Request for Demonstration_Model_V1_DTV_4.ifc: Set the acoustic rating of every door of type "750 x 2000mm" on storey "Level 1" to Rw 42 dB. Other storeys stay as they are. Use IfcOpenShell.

First a look at what the model holds.

```python
import ifcopenshell
import ifcopenshell.util.element

model = ifcopenshell.open("Demonstration_Model_V1_DTV_4.ifc")
print(model.schema)
storey = next(s for s in model.by_type("IfcBuildingStorey") if s.Name == "Level 1")
doors = [e for e in ifcopenshell.util.element.get_decomposition(storey) if e.is_a("IfcDoor")]
seen = {}
for e in doors:
    element_type = ifcopenshell.util.element.get_type(e)
    key = (element_type.Name if element_type != e and element_type else None, ifcopenshell.util.element.get_pset(e, "Pset_DoorCommon", "AcousticRating"))
    seen[key] = seen.get(key, 0) + 1
for (name, value), count in sorted(seen.items(), key=str):
    print(count, "x", name, "|", value)
```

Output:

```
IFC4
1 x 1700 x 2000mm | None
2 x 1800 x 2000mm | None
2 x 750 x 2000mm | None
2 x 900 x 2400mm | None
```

```python
import ifcopenshell
import ifcopenshell.api.pset
import ifcopenshell.util.element

model = ifcopenshell.open("Demonstration_Model_V1_DTV_4.ifc")

storey = next(s for s in model.by_type("IfcBuildingStorey") if s.Name == "Level 1")
doors = [e for e in ifcopenshell.util.element.get_decomposition(storey) if e.is_a("IfcDoor")]

count = 0
for e in doors:
    element_type = ifcopenshell.util.element.get_type(e)
    if element_type in (None, e) or element_type.Name != "750 x 2000mm":
        continue
    # add_pset returns the element's existing set when there is one.
    pset = ifcopenshell.api.pset.add_pset(model, product=e, name="Pset_DoorCommon")
    ifcopenshell.api.pset.edit_pset(model, pset=pset, properties={"AcousticRating": "Rw 42 dB"})
    count += 1

print(count, "doors updated")

model.write("Demonstration_Model_V1_DTV_4_edited.ifc")
```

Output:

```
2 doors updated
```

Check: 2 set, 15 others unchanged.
